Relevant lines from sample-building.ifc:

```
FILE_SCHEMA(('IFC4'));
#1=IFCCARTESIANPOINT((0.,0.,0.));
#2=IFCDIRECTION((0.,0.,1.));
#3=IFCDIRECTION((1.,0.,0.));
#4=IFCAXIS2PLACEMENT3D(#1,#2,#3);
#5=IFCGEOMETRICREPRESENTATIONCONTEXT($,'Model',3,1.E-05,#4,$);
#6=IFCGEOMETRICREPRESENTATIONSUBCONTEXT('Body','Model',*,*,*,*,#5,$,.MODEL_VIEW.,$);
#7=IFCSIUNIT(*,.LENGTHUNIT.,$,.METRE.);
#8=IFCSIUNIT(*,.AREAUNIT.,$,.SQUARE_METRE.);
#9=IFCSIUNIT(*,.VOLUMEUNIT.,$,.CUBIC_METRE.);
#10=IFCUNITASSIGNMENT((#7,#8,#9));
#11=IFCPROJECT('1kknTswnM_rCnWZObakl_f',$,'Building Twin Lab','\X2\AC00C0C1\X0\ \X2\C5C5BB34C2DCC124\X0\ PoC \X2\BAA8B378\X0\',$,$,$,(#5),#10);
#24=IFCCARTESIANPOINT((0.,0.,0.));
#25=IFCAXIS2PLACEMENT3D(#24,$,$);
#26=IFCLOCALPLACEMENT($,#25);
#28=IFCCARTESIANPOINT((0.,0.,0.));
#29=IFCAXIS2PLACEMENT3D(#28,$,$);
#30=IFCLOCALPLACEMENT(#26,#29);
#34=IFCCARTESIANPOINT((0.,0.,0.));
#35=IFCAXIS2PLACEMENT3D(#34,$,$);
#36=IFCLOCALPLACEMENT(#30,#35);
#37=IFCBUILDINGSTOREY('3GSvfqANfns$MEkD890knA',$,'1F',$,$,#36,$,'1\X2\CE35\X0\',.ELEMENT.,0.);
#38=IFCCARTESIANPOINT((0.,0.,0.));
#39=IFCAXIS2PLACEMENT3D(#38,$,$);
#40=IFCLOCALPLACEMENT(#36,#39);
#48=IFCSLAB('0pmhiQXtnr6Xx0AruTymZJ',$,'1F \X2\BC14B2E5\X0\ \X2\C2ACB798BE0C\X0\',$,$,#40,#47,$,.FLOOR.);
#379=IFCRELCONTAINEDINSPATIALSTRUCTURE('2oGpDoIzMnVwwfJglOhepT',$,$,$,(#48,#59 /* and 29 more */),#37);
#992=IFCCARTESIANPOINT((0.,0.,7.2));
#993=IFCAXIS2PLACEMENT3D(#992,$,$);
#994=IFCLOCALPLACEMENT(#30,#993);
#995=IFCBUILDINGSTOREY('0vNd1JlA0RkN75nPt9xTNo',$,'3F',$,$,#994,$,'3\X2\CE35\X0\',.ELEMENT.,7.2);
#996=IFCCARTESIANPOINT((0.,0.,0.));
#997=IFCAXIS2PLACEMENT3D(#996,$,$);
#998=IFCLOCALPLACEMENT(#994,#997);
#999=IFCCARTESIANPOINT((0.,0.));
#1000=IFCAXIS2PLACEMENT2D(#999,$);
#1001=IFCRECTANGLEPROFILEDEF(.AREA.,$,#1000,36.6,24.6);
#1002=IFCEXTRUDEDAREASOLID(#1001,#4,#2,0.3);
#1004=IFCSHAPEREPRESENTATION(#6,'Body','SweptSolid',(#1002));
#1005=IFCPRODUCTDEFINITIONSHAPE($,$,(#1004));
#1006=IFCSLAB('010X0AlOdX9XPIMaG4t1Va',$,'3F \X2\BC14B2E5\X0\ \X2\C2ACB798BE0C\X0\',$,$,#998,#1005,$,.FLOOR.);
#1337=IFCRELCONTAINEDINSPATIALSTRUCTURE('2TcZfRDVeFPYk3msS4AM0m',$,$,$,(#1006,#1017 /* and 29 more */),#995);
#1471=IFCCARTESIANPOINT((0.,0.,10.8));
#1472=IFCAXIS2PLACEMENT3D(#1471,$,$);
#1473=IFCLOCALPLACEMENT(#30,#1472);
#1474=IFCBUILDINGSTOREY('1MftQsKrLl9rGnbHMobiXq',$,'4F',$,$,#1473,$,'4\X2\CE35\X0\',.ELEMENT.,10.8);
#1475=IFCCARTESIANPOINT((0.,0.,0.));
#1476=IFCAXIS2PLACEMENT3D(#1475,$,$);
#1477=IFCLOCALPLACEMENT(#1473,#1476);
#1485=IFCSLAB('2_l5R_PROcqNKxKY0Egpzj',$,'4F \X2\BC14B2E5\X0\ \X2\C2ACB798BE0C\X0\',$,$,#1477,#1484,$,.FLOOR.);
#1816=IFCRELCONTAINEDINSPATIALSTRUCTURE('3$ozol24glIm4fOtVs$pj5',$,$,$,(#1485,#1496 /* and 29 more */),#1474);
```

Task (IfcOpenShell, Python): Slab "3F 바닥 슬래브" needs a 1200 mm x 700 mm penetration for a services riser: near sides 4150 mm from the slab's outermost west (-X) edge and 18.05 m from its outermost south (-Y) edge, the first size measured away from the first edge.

```python
import numpy as np
import ifcopenshell
import ifcopenshell.api.feature
import ifcopenshell.api.geometry
import ifcopenshell.api.root
import ifcopenshell.geom
import ifcopenshell.util.placement
import ifcopenshell.util.representation
import ifcopenshell.util.shape
import ifcopenshell.util.unit

model = ifcopenshell.open("sample-building.ifc")
unit_scale = ifcopenshell.util.unit.calculate_unit_scale(model)
settings = ifcopenshell.geom.settings()


def volume(element):
    """Net volume in cubic metres, openings subtracted."""
    shape = ifcopenshell.geom.create_shape(settings, element)
    return ifcopenshell.util.shape.get_volume(shape.geometry)


slab = model.by_id(1006)
before = volume(slab)

# Extent in the slab's own axes, in metres. The edges named are its -X and -Y sides.
slab_shape = ifcopenshell.geom.create_shape(settings, slab)
vertices = ifcopenshell.util.shape.get_vertices(slab_shape.geometry)
x_min, y_min, bottom = vertices.min(axis=0)
top = vertices[:, 2].max()

opening = ifcopenshell.api.root.create_entity(model, ifc_class="IfcOpeningElement", name="Services riser opening", predefined_type="OPENING")
context = ifcopenshell.util.representation.get_context(model, "Model", "Body", "MODEL_VIEW")
width, depth = 1.2, 0.7
outline = [(0.0, 0.0), (width, 0.0), (width, depth), (0.0, depth), (0.0, 0.0)]
# Overshoot both faces by 50 mm so the cut is clean.
shape = ifcopenshell.api.geometry.add_slab_representation(
    model, context=context, depth=top - bottom + 0.1, polyline=outline
)
ifcopenshell.api.geometry.assign_representation(model, product=opening, representation=shape)

matrix = ifcopenshell.util.placement.get_local_placement(slab.ObjectPlacement)
matrix[:, 3] = matrix @ np.append(np.array([x_min + 4.15, y_min + 18.05, bottom - 0.05]) / unit_scale, 1.0)
ifcopenshell.api.geometry.edit_object_placement(model, product=opening, matrix=matrix, is_si=False)
ifcopenshell.api.feature.add_feature(model, feature=opening, element=slab)

after = volume(slab)

print(f"slab volume {before:.3f} -> {after:.3f} m3")

model.write("sample-building_rev.ifc")
```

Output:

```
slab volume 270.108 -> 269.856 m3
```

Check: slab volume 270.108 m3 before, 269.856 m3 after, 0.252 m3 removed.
